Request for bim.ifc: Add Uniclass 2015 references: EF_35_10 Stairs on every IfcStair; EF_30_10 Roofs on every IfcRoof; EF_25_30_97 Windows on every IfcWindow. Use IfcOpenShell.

First a look at what the model holds.

```python
import ifcopenshell

model = ifcopenshell.open("bim.ifc")
print(model.schema)
print("classifications:", [c.Name for c in model.by_type("IfcClassification")])
for ifc_class in ("IfcDoor", "IfcRoof", "IfcStair", "IfcWall", "IfcWindow"):
    print(ifc_class, len(model.by_type(ifc_class)))
```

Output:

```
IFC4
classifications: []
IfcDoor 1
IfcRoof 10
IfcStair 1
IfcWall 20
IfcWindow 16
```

```python
import ifcopenshell
import ifcopenshell.api.classification

model = ifcopenshell.open("bim.ifc")

system = ifcopenshell.api.classification.add_classification(model, classification="Uniclass 2015")

codes = {
    "IfcStair": ("EF_35_10", "Stairs"),
    "IfcRoof": ("EF_30_10", "Roofs"),
    "IfcWindow": ("EF_25_30_97", "Windows"),
}
for ifc_class, (code, name) in codes.items():
    products = model.by_type(ifc_class)
    ifcopenshell.api.classification.add_reference(
        model, products=products, classification=system, identification=code, name=name
    )
    print(code, len(products))

model.write("bim_rev.ifc")
```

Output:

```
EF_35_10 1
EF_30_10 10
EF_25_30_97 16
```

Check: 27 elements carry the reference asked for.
